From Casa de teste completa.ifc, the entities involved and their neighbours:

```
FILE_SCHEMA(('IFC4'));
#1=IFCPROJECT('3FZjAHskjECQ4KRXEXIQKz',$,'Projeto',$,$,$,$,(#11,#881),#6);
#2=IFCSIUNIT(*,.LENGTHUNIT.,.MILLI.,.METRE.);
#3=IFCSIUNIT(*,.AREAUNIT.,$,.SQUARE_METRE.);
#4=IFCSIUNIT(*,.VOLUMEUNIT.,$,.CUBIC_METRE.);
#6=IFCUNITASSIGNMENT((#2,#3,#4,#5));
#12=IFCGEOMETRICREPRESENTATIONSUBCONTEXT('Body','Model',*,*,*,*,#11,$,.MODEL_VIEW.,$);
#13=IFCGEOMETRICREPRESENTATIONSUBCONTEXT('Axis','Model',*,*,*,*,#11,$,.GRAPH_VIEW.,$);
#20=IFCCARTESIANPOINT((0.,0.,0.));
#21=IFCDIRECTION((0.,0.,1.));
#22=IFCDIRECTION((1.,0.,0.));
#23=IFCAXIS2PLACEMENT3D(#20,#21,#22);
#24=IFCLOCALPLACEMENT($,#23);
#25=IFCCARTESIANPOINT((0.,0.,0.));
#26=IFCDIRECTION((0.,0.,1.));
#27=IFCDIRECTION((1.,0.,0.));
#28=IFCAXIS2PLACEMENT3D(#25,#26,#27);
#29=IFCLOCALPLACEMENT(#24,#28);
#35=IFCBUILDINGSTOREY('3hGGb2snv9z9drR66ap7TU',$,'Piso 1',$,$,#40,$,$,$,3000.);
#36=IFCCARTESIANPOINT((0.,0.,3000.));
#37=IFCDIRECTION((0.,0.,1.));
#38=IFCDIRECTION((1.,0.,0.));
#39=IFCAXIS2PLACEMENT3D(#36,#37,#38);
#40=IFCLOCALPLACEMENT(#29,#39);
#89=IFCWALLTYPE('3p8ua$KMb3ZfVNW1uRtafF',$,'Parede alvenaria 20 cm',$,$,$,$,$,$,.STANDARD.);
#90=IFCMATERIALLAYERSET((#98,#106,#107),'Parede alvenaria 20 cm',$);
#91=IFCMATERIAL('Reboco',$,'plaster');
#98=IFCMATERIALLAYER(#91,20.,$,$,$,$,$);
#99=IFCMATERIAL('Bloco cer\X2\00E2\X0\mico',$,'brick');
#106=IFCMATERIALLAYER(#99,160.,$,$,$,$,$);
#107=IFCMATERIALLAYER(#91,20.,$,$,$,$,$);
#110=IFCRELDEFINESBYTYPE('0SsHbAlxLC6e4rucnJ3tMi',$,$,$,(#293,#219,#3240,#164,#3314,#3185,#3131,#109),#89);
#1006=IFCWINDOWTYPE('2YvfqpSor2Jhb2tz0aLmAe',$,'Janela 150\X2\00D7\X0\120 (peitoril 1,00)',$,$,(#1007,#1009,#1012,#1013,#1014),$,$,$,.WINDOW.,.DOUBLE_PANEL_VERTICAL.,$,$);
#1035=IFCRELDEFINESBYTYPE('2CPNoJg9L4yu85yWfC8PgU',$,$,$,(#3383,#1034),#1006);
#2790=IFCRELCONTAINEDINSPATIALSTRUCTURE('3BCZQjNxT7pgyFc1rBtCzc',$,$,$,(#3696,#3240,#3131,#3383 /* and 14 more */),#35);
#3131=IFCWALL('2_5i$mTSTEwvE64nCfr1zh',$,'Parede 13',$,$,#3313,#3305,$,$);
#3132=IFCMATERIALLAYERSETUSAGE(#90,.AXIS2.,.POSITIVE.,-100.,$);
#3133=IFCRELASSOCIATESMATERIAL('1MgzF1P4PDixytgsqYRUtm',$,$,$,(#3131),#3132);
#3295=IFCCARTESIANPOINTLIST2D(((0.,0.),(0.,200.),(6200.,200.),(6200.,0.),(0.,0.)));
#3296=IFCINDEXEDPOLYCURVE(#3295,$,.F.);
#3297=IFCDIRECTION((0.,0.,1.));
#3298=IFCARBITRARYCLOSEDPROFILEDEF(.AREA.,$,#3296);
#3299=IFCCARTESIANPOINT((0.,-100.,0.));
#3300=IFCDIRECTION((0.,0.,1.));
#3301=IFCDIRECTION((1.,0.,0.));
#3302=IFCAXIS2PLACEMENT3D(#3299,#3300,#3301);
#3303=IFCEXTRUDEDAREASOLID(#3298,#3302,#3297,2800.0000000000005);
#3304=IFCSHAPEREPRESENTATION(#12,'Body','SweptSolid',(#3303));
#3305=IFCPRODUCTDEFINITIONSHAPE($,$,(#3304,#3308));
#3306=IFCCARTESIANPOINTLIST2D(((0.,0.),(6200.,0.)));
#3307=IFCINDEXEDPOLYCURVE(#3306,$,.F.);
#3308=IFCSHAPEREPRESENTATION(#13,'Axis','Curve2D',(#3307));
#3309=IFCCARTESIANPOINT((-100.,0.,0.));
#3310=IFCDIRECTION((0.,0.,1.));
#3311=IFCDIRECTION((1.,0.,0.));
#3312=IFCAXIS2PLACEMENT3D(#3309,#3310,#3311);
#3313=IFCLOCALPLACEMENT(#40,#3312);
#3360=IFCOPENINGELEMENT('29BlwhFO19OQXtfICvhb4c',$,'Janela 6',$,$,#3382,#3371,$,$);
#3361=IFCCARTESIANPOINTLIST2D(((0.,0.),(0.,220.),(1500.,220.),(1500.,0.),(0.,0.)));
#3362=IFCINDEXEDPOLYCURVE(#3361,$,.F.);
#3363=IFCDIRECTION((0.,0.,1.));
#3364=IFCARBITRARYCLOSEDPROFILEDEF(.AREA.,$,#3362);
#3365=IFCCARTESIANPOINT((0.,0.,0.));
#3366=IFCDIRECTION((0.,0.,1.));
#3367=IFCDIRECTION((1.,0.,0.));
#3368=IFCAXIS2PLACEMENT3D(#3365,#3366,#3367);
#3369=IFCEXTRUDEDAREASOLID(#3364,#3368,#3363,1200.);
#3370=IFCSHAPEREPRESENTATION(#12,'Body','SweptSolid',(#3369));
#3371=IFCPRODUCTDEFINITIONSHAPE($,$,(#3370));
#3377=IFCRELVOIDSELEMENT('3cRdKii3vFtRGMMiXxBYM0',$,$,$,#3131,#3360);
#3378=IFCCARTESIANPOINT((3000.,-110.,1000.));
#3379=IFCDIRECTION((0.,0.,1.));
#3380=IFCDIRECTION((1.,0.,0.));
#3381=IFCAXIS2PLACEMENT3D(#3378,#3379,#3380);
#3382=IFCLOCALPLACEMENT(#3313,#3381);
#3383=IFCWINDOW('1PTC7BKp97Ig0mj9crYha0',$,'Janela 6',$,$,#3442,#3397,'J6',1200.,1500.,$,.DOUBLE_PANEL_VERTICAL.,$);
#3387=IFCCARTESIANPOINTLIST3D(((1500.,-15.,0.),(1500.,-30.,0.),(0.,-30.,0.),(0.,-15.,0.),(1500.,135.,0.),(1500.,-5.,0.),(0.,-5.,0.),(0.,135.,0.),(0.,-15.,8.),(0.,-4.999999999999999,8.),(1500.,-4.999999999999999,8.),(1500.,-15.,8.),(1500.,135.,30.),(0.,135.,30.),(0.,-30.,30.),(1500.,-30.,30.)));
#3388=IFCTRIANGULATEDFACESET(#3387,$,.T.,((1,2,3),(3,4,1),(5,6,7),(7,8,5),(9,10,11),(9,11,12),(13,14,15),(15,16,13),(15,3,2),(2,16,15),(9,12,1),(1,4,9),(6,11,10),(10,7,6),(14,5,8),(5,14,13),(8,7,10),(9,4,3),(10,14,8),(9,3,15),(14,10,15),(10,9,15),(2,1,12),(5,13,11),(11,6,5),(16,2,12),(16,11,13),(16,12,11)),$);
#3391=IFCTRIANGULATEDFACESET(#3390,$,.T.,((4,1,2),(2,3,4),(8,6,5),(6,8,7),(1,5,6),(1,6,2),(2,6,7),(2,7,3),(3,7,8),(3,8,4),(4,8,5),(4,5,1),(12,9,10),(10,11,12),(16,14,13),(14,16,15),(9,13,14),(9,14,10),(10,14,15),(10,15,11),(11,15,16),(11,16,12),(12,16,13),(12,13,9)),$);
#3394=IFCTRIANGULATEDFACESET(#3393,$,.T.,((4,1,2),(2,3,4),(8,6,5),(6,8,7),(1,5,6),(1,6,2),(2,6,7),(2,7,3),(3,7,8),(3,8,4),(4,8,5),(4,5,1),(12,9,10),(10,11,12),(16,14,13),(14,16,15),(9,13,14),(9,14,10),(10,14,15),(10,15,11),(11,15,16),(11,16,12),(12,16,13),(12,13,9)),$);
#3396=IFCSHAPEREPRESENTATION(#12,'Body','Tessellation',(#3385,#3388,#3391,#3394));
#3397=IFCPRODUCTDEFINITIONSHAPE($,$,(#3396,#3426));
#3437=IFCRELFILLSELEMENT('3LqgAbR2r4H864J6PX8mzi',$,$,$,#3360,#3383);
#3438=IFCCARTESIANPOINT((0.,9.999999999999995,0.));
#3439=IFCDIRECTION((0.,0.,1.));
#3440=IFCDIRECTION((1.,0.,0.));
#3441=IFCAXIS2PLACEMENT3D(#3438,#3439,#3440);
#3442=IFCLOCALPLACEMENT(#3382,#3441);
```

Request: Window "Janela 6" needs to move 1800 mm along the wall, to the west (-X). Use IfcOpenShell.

```python
import ifcopenshell
import ifcopenshell.api.geometry
import ifcopenshell.util.placement
import ifcopenshell.util.unit

model = ifcopenshell.open("Casa de teste completa.ifc")
unit_scale = ifcopenshell.util.unit.calculate_unit_scale(model)

window = model.by_id(3383)
opening = window.FillsVoids[0].RelatingOpeningElement
wall = opening.VoidsElements[0].RelatingBuildingElement

wall_matrix = ifcopenshell.util.placement.get_local_placement(wall.ObjectPlacement)
shift = wall_matrix[:3, 0] * -1.8 / unit_scale
before = ifcopenshell.util.placement.get_local_placement(window.ObjectPlacement)[:3, 3].copy()

# The window is placed relative to its opening, so it follows when the opening moves.
matrix = ifcopenshell.util.placement.get_local_placement(opening.ObjectPlacement)
matrix[:3, 3] += shift
ifcopenshell.api.geometry.edit_object_placement(
    model, product=opening, matrix=matrix, is_si=False, should_transform_children=True
)

after = ifcopenshell.util.placement.get_local_placement(window.ObjectPlacement)[:3, 3]
print("window moved by", (after - before).round(3) + 0.0)

model.write("Casa de teste completa-out.ifc")
```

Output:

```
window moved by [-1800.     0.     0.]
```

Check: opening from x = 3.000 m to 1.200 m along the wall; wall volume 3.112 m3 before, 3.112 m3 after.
